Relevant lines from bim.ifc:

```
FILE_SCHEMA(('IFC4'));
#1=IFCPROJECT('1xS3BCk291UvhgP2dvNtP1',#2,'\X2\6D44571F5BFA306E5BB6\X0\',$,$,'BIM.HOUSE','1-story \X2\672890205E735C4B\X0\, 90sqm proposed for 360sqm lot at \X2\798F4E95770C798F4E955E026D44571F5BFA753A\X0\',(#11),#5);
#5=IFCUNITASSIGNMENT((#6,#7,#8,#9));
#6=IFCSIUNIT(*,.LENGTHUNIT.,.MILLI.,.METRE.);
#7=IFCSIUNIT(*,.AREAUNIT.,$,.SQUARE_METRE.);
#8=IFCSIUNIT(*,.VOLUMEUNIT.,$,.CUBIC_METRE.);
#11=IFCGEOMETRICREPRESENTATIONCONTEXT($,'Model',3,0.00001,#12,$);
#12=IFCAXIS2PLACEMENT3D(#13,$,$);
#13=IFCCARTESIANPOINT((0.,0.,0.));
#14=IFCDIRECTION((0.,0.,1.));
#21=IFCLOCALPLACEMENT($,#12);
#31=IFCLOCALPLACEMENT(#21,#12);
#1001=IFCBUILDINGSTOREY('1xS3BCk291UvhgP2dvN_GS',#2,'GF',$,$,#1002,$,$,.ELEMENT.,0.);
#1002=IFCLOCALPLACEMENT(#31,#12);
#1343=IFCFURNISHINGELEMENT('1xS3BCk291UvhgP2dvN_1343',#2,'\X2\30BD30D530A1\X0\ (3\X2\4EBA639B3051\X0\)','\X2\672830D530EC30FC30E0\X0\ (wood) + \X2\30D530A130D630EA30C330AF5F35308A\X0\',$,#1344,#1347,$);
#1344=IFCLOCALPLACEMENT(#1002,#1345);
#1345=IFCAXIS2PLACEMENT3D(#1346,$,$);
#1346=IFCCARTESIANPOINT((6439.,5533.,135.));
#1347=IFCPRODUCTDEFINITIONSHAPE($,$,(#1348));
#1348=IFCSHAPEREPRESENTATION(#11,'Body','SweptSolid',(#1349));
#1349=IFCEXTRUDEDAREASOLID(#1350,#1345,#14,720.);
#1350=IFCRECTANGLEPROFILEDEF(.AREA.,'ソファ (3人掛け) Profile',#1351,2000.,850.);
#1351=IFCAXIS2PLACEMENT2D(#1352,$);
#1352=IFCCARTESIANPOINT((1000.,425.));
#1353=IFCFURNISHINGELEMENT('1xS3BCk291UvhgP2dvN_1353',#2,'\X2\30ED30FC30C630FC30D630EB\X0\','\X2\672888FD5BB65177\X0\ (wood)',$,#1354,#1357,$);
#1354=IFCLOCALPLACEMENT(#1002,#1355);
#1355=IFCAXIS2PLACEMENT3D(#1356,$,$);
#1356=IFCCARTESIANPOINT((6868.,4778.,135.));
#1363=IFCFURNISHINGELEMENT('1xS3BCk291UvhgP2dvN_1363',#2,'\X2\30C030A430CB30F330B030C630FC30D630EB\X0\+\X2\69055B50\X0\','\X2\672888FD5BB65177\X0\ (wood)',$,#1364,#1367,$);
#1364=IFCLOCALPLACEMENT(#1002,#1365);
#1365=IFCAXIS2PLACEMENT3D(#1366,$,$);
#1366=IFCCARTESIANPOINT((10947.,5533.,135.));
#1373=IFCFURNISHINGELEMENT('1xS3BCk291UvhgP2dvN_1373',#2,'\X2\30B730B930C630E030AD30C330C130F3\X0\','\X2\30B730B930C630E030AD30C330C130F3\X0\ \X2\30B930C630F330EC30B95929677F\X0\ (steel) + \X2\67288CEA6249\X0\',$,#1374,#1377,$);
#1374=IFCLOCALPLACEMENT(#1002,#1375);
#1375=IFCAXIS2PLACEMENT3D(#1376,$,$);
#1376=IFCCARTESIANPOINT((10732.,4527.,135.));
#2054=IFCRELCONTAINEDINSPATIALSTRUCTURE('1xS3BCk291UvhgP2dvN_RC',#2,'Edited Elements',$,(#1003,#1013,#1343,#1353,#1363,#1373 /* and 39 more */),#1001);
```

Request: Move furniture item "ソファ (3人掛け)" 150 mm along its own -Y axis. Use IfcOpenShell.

```python
import ifcopenshell
import ifcopenshell.api.geometry
import ifcopenshell.util.placement

model = ifcopenshell.open("bim.ifc")

item = model.by_id(1343)
matrix = ifcopenshell.util.placement.get_local_placement(item.ObjectPlacement)
matrix[:3, 3] -= matrix[:3, 1] * 150.0
ifcopenshell.api.geometry.edit_object_placement(model, product=item, matrix=matrix, is_si=False)

print(ifcopenshell.util.placement.get_local_placement(item.ObjectPlacement).round(3) + 0.0)

model.write("bim-out.ifc")
```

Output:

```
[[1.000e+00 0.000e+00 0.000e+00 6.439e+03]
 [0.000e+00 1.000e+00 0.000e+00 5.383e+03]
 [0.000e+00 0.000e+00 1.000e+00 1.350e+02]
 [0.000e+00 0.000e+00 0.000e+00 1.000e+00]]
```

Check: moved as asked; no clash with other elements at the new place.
